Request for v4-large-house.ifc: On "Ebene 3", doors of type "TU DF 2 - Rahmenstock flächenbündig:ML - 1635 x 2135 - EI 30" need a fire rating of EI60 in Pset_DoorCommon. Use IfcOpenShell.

First a look at what the model holds.

```python
import ifcopenshell
import ifcopenshell.util.element

model = ifcopenshell.open("v4-large-house.ifc")
print(model.schema)
storey = next(s for s in model.by_type("IfcBuildingStorey") if s.Name == "Ebene 3")
doors = [e for e in ifcopenshell.util.element.get_decomposition(storey) if e.is_a("IfcDoor")]
seen = {}
for e in doors:
    element_type = ifcopenshell.util.element.get_type(e)
    key = (element_type.Name if element_type != e and element_type else None, ifcopenshell.util.element.get_pset(e, "Pset_DoorCommon", "FireRating"))
    seen[key] = seen.get(key, 0) + 1
for (name, value), count in sorted(seen.items(), key=str):
    print(count, "x", name, "|", value)
```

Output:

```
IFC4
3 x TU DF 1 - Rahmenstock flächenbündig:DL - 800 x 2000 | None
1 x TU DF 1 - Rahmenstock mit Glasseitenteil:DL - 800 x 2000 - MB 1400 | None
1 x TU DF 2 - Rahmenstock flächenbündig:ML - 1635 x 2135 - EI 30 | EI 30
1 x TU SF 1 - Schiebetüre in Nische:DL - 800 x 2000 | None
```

```python
import ifcopenshell
import ifcopenshell.api.pset
import ifcopenshell.util.element

model = ifcopenshell.open("v4-large-house.ifc")

storey = next(s for s in model.by_type("IfcBuildingStorey") if s.Name == "Ebene 3")
doors = [e for e in ifcopenshell.util.element.get_decomposition(storey) if e.is_a("IfcDoor")]

count = 0
for e in doors:
    element_type = ifcopenshell.util.element.get_type(e)
    if element_type in (None, e) or element_type.Name != "TU DF 2 - Rahmenstock flächenbündig:ML - 1635 x 2135 - EI 30":
        continue
    # add_pset returns the element's existing set when there is one.
    pset = ifcopenshell.api.pset.add_pset(model, product=e, name="Pset_DoorCommon")
    ifcopenshell.api.pset.edit_pset(model, pset=pset, properties={"FireRating": "EI60"})
    count += 1

print(count, "doors updated")

model.write("v4-large-house_v2.ifc")
```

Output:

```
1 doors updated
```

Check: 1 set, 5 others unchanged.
